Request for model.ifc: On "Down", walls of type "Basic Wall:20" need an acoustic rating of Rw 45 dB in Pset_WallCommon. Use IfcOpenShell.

First a look at what the model holds.

```python
import ifcopenshell
import ifcopenshell.util.element

model = ifcopenshell.open("model.ifc")
print(model.schema)
storey = next(s for s in model.by_type("IfcBuildingStorey") if s.Name == "Down")
walls = [e for e in ifcopenshell.util.element.get_decomposition(storey) if e.is_a("IfcWall")]
seen = {}
for e in walls:
    element_type = ifcopenshell.util.element.get_type(e)
    key = (element_type.Name if element_type != e and element_type else None, ifcopenshell.util.element.get_pset(e, "Pset_WallCommon", "AcousticRating"))
    seen[key] = seen.get(key, 0) + 1
for (name, value), count in sorted(seen.items(), key=str):
    print(count, "x", name, "|", value)
```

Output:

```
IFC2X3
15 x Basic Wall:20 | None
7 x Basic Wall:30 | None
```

```python
import ifcopenshell
import ifcopenshell.api.pset
import ifcopenshell.util.element

model = ifcopenshell.open("model.ifc")

storey = next(s for s in model.by_type("IfcBuildingStorey") if s.Name == "Down")
walls = [e for e in ifcopenshell.util.element.get_decomposition(storey) if e.is_a("IfcWall")]

count = 0
for e in walls:
    element_type = ifcopenshell.util.element.get_type(e)
    if element_type in (None, e) or element_type.Name != "Basic Wall:20":
        continue
    # add_pset returns the element's existing set when there is one.
    pset = ifcopenshell.api.pset.add_pset(model, product=e, name="Pset_WallCommon")
    ifcopenshell.api.pset.edit_pset(model, pset=pset, properties={"AcousticRating": "Rw 45 dB"})
    count += 1

print(count, "walls updated")

model.write("model_rev.ifc")
```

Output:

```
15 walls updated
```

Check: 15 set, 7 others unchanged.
